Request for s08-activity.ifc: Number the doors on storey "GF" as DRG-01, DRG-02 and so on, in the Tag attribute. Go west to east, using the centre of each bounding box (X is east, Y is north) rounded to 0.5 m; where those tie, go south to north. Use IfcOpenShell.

First a look at what the model holds.

```python
import ifcopenshell
import ifcopenshell.util.element
import ifcopenshell.util.placement

model = ifcopenshell.open("s08-activity.ifc")
print(model.schema)
storey = next(s for s in model.by_type("IfcBuildingStorey") if s.Name == "GF")
doors = [e for e in ifcopenshell.util.element.get_decomposition(storey) if e.is_a("IfcDoor")]
for e in sorted(doors, key=lambda e: e.id()):
    origin = ifcopenshell.util.placement.get_local_placement(e.ObjectPlacement)[:3, 3]
    print(e.id(), e.Tag, e.Name, origin.round(2) + 0.0, sep=" | ")
```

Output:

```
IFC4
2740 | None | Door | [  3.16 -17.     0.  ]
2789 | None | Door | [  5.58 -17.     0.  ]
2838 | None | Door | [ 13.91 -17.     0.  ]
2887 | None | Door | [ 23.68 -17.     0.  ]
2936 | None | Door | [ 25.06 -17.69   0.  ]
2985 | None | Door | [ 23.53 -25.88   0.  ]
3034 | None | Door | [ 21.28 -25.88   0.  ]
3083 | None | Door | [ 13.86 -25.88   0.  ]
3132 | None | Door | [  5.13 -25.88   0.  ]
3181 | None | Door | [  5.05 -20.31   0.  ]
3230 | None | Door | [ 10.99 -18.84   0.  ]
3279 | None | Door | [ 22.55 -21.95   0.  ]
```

```python
import ifcopenshell
import ifcopenshell.geom
import ifcopenshell.util.element
import ifcopenshell.util.shape

model = ifcopenshell.open("s08-activity.ifc")
settings = ifcopenshell.geom.settings()
settings.set("use-world-coords", True)


def centre(element):
    shape = ifcopenshell.geom.create_shape(settings, element)
    return ifcopenshell.util.shape.get_bbox_centroid(shape.geometry)


storey = next(s for s in model.by_type("IfcBuildingStorey") if s.Name == "GF")
doors = [e for e in ifcopenshell.util.element.get_decomposition(storey) if e.is_a("IfcDoor")]

# Insertion points can sit at a corner or the storey origin, so sort by the geometry (in metres).
centres = {e: centre(e) for e in doors}
doors.sort(key=lambda e: (round(centres[e][0] / 0.5), centres[e][1]))

for i, e in enumerate(doors, start=1):
    number = f"DRG-{i:02d}"
    e.Tag = number
    print(e.id(), number)

model.write("s08-activity-out.ifc")
```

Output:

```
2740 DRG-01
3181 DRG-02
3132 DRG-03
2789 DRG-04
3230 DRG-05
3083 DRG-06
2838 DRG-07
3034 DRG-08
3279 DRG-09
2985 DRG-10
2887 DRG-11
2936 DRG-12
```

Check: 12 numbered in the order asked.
